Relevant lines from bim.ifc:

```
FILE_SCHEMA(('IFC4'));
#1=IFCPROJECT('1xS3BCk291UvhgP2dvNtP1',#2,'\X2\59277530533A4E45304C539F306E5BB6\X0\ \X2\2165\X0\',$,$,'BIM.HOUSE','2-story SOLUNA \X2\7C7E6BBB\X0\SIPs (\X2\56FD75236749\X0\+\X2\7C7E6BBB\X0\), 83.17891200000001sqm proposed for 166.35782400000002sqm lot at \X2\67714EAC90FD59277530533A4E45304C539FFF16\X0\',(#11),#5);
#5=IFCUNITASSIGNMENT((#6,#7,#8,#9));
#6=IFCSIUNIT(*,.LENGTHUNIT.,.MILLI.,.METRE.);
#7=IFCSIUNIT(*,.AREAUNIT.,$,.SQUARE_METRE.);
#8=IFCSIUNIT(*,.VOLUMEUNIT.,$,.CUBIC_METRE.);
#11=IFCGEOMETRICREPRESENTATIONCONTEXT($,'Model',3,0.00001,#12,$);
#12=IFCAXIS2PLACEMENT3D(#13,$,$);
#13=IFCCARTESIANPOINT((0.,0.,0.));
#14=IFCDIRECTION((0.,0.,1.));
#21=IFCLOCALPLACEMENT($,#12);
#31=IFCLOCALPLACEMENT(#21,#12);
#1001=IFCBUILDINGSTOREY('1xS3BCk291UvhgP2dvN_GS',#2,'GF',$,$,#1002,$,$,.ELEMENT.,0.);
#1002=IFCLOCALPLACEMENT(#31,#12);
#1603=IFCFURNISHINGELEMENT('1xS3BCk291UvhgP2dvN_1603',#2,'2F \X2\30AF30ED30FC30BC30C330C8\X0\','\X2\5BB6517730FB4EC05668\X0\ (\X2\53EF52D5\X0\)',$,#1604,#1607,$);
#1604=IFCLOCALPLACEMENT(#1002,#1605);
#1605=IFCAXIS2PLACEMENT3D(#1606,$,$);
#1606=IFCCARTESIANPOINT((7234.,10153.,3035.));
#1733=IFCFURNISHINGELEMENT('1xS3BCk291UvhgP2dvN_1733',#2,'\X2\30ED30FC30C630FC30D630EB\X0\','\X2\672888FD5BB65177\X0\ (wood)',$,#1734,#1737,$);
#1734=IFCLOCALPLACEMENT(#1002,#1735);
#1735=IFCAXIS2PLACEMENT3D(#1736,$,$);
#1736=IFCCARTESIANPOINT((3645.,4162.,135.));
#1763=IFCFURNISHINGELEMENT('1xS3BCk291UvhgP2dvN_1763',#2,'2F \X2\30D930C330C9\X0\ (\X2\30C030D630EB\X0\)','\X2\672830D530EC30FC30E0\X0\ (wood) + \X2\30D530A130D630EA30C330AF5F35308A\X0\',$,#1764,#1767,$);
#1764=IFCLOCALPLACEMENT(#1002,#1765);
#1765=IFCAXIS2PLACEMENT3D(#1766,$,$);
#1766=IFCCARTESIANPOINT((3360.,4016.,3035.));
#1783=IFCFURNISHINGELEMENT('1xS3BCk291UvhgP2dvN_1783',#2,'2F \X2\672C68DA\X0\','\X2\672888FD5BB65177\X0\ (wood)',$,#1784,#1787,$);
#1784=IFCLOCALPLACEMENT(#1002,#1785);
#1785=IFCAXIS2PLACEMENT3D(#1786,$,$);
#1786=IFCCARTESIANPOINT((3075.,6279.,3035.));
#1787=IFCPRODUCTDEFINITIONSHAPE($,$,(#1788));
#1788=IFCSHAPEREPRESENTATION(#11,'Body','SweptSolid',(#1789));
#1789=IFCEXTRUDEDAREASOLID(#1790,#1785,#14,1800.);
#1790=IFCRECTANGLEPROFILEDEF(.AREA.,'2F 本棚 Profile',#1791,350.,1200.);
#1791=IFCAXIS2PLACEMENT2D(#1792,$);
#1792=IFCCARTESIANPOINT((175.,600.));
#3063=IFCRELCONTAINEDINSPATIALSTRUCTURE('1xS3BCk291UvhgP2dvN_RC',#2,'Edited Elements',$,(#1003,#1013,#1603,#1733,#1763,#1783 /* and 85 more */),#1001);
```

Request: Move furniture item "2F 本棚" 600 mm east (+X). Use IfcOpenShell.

```python
import ifcopenshell
import ifcopenshell.api.geometry
import ifcopenshell.util.placement
import ifcopenshell.util.unit

model = ifcopenshell.open("bim.ifc")
unit_scale = ifcopenshell.util.unit.calculate_unit_scale(model)

item = model.by_id(1783)
matrix = ifcopenshell.util.placement.get_local_placement(item.ObjectPlacement)
matrix[0, 3] += 0.6 / unit_scale
ifcopenshell.api.geometry.edit_object_placement(model, product=item, matrix=matrix, is_si=False)

print(ifcopenshell.util.placement.get_local_placement(item.ObjectPlacement).round(3) + 0.0)

model.write("bim-out.ifc")
```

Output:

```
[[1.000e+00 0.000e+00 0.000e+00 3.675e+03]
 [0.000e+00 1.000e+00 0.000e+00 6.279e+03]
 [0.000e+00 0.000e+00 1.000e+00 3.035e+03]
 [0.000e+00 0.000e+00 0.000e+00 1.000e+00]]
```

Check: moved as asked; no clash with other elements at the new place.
